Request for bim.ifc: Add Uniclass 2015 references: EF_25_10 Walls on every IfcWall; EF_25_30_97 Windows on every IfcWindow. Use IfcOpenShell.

First a look at what the model holds.

```python
import ifcopenshell

model = ifcopenshell.open("bim.ifc")
print(model.schema)
print("classifications:", [c.Name for c in model.by_type("IfcClassification")])
for ifc_class in ("IfcDoor", "IfcRoof", "IfcStair", "IfcWall", "IfcWindow"):
    print(ifc_class, len(model.by_type(ifc_class)))
```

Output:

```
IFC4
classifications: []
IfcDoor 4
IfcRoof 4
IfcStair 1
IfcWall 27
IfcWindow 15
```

```python
import ifcopenshell
import ifcopenshell.api.classification

model = ifcopenshell.open("bim.ifc")

system = ifcopenshell.api.classification.add_classification(model, classification="Uniclass 2015")

codes = {
    "IfcWall": ("EF_25_10", "Walls"),
    "IfcWindow": ("EF_25_30_97", "Windows"),
}
for ifc_class, (code, name) in codes.items():
    products = model.by_type(ifc_class)
    ifcopenshell.api.classification.add_reference(
        model, products=products, classification=system, identification=code, name=name
    )
    print(code, len(products))

model.write("bim_updated.ifc")
```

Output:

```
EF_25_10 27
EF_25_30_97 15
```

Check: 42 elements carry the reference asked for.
